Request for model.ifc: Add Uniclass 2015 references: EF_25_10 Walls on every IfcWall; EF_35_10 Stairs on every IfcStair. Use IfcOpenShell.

First a look at what the model holds.

```python
import ifcopenshell

model = ifcopenshell.open("model.ifc")
print(model.schema)
print("classifications:", [c.Name for c in model.by_type("IfcClassification")])
for ifc_class in ("IfcDoor", "IfcRoof", "IfcStair", "IfcWall", "IfcWindow"):
    print(ifc_class, len(model.by_type(ifc_class)))
```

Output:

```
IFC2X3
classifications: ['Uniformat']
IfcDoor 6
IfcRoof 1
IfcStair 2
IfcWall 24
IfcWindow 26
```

```python
import ifcopenshell
import ifcopenshell.api.classification

model = ifcopenshell.open("model.ifc")

# IFC2X3 requires Source and Edition and has no link from the project to the system.
system = model.create_entity("IfcClassification", Source="NBS", Edition="2015", Name="Uniclass 2015")

codes = {
    "IfcWall": ("EF_25_10", "Walls"),
    "IfcStair": ("EF_35_10", "Stairs"),
}
for ifc_class, (code, name) in codes.items():
    products = model.by_type(ifc_class)
    ifcopenshell.api.classification.add_reference(
        model, products=products, classification=system, identification=code, name=name
    )
    print(code, len(products))

model.write("model-out.ifc")
```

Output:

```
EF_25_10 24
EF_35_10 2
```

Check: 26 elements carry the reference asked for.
